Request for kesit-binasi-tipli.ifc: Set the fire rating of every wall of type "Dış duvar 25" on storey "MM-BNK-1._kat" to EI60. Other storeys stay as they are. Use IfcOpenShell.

First a look at what the model holds.

```python
import ifcopenshell
import ifcopenshell.util.element

model = ifcopenshell.open("kesit-binasi-tipli.ifc")
print(model.schema)
storey = next(s for s in model.by_type("IfcBuildingStorey") if s.Name == "MM-BNK-1._kat")
walls = [e for e in ifcopenshell.util.element.get_decomposition(storey) if e.is_a("IfcWall")]
seen = {}
for e in walls:
    element_type = ifcopenshell.util.element.get_type(e)
    key = (element_type.Name if element_type != e and element_type else None, ifcopenshell.util.element.get_pset(e, "Pset_WallCommon", "FireRating"))
    seen[key] = seen.get(key, 0) + 1
for (name, value), count in sorted(seen.items(), key=str):
    print(count, "x", name, "|", value)
```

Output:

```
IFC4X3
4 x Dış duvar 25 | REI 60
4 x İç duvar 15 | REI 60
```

```python
import ifcopenshell
import ifcopenshell.api.pset
import ifcopenshell.util.element

model = ifcopenshell.open("kesit-binasi-tipli.ifc")

storey = next(s for s in model.by_type("IfcBuildingStorey") if s.Name == "MM-BNK-1._kat")
walls = [e for e in ifcopenshell.util.element.get_decomposition(storey) if e.is_a("IfcWall")]

count = 0
for e in walls:
    element_type = ifcopenshell.util.element.get_type(e)
    if element_type in (None, e) or element_type.Name != "Dış duvar 25":
        continue
    # add_pset returns the element's existing set when there is one.
    pset = ifcopenshell.api.pset.add_pset(model, product=e, name="Pset_WallCommon")
    ifcopenshell.api.pset.edit_pset(model, pset=pset, properties={"FireRating": "EI60"})
    count += 1

print(count, "walls updated")

model.write("kesit-binasi-tipli_rev.ifc")
```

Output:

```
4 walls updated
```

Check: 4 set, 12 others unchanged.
